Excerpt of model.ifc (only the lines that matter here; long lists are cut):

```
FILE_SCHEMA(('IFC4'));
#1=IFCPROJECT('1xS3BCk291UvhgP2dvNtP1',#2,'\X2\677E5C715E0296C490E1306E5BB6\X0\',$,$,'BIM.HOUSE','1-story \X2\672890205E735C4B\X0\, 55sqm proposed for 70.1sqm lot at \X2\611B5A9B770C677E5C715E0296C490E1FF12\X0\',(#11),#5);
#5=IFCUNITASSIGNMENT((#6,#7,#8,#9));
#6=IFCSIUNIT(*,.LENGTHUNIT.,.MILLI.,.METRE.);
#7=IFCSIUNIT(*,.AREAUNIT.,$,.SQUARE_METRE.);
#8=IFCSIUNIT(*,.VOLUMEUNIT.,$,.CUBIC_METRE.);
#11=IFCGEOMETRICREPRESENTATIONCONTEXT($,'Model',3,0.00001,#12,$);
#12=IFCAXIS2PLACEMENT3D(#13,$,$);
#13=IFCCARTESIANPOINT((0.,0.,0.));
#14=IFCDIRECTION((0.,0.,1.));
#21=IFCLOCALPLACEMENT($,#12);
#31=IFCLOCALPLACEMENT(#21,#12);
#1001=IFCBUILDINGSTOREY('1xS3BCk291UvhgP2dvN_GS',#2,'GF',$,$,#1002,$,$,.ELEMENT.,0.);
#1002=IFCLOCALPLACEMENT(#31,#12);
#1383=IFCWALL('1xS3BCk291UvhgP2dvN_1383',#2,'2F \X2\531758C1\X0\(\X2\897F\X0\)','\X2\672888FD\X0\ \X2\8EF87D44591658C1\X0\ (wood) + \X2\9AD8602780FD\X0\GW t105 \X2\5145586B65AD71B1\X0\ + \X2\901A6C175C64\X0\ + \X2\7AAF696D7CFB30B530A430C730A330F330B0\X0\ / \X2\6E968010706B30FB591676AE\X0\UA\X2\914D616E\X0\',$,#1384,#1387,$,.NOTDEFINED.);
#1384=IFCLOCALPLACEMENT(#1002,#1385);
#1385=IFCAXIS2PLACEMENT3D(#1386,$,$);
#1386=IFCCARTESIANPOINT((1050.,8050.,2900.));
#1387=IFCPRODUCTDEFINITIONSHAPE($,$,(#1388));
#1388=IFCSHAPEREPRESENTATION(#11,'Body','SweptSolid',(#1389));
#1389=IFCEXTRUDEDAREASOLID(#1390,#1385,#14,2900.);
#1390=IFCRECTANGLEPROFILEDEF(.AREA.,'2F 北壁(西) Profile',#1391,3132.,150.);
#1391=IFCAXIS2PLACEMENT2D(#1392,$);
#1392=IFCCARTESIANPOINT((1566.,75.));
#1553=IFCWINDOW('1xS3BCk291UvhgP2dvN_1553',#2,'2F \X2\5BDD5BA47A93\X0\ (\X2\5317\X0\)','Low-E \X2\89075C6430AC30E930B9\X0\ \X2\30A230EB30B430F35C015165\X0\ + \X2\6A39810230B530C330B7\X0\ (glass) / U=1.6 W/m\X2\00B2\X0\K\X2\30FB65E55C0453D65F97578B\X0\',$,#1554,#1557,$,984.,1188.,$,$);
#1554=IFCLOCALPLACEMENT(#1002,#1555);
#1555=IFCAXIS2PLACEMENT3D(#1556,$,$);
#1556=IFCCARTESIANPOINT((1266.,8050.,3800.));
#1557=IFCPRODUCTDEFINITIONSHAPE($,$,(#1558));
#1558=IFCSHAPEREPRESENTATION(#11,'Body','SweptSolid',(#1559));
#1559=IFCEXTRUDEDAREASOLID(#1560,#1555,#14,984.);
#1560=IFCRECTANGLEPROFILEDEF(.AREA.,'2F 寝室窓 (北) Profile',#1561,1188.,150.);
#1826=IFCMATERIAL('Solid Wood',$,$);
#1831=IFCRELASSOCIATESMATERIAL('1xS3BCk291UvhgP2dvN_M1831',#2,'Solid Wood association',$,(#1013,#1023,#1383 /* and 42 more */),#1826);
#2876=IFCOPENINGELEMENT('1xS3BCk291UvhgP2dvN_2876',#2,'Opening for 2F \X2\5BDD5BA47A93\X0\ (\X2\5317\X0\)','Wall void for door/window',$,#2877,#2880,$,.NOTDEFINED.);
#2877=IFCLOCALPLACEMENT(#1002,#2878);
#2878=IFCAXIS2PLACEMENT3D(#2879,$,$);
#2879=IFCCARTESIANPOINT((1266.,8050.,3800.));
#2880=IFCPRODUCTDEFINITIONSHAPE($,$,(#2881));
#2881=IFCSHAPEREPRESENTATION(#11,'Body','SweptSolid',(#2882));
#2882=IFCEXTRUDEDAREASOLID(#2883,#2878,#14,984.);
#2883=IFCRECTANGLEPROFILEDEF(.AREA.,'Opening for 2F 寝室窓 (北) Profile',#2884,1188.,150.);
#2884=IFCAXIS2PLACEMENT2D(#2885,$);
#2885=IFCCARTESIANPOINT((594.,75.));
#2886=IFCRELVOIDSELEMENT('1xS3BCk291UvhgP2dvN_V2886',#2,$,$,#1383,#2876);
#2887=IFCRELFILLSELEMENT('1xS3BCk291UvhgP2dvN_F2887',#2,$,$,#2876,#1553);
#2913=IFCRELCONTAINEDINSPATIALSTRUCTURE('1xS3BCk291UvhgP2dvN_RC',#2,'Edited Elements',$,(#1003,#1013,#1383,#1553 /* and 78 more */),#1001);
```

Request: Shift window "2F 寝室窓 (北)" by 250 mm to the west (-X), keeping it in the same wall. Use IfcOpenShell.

```python
import ifcopenshell
import ifcopenshell.api.geometry
import ifcopenshell.util.placement

model = ifcopenshell.open("model.ifc")

window = model.by_id(1553)
opening = window.FillsVoids[0].RelatingOpeningElement
wall = opening.VoidsElements[0].RelatingBuildingElement

wall_matrix = ifcopenshell.util.placement.get_local_placement(wall.ObjectPlacement)
shift = wall_matrix[:3, 0] * -250.0
before = ifcopenshell.util.placement.get_local_placement(window.ObjectPlacement)[:3, 3].copy()

# The window is not placed relative to its opening, so move both.
for product in (opening, window):
    matrix = ifcopenshell.util.placement.get_local_placement(product.ObjectPlacement)
    matrix[:3, 3] += shift
    ifcopenshell.api.geometry.edit_object_placement(model, product=product, matrix=matrix, is_si=False)

after = ifcopenshell.util.placement.get_local_placement(window.ObjectPlacement)[:3, 3]
print("window moved by", (after - before).round(3) + 0.0)

model.write("model_edited.ifc")
```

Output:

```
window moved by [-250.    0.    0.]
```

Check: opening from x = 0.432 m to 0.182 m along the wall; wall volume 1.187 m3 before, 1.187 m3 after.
